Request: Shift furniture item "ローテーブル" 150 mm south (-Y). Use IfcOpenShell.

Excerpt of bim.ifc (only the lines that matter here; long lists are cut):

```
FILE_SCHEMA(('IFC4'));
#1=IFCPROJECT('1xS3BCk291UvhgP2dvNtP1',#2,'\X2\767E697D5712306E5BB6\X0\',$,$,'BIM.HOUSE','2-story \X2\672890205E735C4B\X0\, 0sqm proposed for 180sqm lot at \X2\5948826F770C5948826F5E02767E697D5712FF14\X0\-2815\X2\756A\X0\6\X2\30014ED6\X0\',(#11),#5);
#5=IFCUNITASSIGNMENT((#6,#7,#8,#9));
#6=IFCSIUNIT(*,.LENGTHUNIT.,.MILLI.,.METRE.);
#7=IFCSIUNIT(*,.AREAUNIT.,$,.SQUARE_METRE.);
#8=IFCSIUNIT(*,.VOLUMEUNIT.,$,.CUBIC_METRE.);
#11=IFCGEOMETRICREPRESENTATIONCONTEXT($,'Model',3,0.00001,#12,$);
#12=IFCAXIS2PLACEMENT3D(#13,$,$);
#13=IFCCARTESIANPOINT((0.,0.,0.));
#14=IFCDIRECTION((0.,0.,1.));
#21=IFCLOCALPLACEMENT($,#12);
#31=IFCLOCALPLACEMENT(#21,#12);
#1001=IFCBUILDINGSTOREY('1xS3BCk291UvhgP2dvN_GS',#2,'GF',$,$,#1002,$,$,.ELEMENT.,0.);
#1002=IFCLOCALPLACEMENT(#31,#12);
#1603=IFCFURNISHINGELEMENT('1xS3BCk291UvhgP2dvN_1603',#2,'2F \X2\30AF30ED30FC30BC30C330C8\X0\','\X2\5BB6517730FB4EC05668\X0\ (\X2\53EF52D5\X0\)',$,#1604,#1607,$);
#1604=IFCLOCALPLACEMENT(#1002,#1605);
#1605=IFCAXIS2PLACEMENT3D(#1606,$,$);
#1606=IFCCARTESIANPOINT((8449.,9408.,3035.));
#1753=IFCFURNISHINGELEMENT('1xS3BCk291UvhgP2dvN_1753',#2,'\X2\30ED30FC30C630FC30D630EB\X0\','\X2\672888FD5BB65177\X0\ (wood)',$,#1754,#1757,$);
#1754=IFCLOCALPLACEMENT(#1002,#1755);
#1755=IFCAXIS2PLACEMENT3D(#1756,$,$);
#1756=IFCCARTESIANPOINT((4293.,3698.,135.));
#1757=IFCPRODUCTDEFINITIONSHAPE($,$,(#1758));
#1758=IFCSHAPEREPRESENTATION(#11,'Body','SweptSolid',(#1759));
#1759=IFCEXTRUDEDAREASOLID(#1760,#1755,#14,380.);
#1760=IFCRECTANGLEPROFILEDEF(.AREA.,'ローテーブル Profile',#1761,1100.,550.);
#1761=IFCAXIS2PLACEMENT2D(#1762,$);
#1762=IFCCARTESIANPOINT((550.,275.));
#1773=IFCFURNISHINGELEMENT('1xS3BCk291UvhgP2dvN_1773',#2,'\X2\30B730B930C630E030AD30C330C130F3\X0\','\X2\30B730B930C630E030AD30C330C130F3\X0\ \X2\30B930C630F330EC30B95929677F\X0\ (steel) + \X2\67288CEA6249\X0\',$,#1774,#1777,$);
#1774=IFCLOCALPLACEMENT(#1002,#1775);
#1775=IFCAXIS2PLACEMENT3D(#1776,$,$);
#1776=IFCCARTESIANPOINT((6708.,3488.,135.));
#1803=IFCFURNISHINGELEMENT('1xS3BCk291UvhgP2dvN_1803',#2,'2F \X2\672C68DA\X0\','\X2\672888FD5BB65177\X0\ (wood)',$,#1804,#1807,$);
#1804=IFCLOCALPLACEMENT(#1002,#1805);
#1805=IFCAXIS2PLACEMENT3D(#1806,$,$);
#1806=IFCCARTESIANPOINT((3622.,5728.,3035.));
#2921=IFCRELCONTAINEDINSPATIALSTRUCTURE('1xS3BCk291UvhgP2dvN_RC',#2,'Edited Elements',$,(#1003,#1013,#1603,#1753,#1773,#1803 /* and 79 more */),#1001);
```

```python
import ifcopenshell
import ifcopenshell.api.geometry
import ifcopenshell.util.placement
import ifcopenshell.util.unit

model = ifcopenshell.open("bim.ifc")
unit_scale = ifcopenshell.util.unit.calculate_unit_scale(model)

item = model.by_guid("1xS3BCk291UvhgP2dvN_1753")
matrix = ifcopenshell.util.placement.get_local_placement(item.ObjectPlacement)
matrix[1, 3] -= 0.15 / unit_scale
ifcopenshell.api.geometry.edit_object_placement(model, product=item, matrix=matrix, is_si=False)

print(ifcopenshell.util.placement.get_local_placement(item.ObjectPlacement).round(3) + 0.0)

model.write("bim-out.ifc")
```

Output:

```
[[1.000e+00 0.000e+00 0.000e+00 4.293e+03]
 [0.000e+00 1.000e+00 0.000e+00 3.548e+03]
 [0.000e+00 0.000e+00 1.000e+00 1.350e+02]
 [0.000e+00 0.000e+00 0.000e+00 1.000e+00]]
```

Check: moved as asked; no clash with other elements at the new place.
